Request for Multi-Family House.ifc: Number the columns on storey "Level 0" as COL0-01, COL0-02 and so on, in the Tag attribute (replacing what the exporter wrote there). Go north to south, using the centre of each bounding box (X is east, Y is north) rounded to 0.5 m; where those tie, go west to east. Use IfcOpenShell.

First a look at what the model holds.

```python
import ifcopenshell
import ifcopenshell.util.element
import ifcopenshell.util.placement

model = ifcopenshell.open("Multi-Family House.ifc")
print(model.schema)
storey = next(s for s in model.by_type("IfcBuildingStorey") if s.Name == "Level 0")
columns = [e for e in ifcopenshell.util.element.get_decomposition(storey) if e.is_a("IfcColumn")]
for e in sorted(columns, key=lambda e: e.id()):
    origin = ifcopenshell.util.placement.get_local_placement(e.ObjectPlacement)[:3, 3]
    print(e.id(), e.Tag, e.Name, origin.round(2) + 0.0, sep=" | ")
```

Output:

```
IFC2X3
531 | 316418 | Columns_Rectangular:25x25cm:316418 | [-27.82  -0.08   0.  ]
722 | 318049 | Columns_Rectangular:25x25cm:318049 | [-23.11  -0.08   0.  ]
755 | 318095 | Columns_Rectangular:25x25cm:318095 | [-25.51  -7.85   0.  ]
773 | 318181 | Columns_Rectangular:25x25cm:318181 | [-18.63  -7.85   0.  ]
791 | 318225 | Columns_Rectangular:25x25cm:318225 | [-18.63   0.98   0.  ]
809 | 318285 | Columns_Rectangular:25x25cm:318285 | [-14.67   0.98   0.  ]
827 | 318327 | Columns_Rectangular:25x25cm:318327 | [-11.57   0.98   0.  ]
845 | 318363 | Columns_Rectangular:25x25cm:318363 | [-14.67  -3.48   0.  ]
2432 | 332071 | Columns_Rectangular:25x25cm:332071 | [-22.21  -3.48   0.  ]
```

```python
import ifcopenshell
import ifcopenshell.geom
import ifcopenshell.util.element
import ifcopenshell.util.shape

model = ifcopenshell.open("Multi-Family House.ifc")
settings = ifcopenshell.geom.settings()
settings.set("use-world-coords", True)


def centre(element):
    shape = ifcopenshell.geom.create_shape(settings, element)
    return ifcopenshell.util.shape.get_bbox_centroid(shape.geometry)


storey = next(s for s in model.by_type("IfcBuildingStorey") if s.Name == "Level 0")
columns = [e for e in ifcopenshell.util.element.get_decomposition(storey) if e.is_a("IfcColumn")]

# Insertion points can sit at a corner or the storey origin, so sort by the geometry (in metres).
centres = {e: centre(e) for e in columns}
columns.sort(key=lambda e: (-round(centres[e][1] / 0.5), centres[e][0]))

for i, e in enumerate(columns, start=1):
    number = f"COL0-{i:02d}"
    e.Tag = number
    print(e.id(), number)

model.write("Multi-Family House_edited.ifc")
```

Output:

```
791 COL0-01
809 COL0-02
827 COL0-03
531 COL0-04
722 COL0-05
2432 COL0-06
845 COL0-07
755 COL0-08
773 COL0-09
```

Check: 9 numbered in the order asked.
